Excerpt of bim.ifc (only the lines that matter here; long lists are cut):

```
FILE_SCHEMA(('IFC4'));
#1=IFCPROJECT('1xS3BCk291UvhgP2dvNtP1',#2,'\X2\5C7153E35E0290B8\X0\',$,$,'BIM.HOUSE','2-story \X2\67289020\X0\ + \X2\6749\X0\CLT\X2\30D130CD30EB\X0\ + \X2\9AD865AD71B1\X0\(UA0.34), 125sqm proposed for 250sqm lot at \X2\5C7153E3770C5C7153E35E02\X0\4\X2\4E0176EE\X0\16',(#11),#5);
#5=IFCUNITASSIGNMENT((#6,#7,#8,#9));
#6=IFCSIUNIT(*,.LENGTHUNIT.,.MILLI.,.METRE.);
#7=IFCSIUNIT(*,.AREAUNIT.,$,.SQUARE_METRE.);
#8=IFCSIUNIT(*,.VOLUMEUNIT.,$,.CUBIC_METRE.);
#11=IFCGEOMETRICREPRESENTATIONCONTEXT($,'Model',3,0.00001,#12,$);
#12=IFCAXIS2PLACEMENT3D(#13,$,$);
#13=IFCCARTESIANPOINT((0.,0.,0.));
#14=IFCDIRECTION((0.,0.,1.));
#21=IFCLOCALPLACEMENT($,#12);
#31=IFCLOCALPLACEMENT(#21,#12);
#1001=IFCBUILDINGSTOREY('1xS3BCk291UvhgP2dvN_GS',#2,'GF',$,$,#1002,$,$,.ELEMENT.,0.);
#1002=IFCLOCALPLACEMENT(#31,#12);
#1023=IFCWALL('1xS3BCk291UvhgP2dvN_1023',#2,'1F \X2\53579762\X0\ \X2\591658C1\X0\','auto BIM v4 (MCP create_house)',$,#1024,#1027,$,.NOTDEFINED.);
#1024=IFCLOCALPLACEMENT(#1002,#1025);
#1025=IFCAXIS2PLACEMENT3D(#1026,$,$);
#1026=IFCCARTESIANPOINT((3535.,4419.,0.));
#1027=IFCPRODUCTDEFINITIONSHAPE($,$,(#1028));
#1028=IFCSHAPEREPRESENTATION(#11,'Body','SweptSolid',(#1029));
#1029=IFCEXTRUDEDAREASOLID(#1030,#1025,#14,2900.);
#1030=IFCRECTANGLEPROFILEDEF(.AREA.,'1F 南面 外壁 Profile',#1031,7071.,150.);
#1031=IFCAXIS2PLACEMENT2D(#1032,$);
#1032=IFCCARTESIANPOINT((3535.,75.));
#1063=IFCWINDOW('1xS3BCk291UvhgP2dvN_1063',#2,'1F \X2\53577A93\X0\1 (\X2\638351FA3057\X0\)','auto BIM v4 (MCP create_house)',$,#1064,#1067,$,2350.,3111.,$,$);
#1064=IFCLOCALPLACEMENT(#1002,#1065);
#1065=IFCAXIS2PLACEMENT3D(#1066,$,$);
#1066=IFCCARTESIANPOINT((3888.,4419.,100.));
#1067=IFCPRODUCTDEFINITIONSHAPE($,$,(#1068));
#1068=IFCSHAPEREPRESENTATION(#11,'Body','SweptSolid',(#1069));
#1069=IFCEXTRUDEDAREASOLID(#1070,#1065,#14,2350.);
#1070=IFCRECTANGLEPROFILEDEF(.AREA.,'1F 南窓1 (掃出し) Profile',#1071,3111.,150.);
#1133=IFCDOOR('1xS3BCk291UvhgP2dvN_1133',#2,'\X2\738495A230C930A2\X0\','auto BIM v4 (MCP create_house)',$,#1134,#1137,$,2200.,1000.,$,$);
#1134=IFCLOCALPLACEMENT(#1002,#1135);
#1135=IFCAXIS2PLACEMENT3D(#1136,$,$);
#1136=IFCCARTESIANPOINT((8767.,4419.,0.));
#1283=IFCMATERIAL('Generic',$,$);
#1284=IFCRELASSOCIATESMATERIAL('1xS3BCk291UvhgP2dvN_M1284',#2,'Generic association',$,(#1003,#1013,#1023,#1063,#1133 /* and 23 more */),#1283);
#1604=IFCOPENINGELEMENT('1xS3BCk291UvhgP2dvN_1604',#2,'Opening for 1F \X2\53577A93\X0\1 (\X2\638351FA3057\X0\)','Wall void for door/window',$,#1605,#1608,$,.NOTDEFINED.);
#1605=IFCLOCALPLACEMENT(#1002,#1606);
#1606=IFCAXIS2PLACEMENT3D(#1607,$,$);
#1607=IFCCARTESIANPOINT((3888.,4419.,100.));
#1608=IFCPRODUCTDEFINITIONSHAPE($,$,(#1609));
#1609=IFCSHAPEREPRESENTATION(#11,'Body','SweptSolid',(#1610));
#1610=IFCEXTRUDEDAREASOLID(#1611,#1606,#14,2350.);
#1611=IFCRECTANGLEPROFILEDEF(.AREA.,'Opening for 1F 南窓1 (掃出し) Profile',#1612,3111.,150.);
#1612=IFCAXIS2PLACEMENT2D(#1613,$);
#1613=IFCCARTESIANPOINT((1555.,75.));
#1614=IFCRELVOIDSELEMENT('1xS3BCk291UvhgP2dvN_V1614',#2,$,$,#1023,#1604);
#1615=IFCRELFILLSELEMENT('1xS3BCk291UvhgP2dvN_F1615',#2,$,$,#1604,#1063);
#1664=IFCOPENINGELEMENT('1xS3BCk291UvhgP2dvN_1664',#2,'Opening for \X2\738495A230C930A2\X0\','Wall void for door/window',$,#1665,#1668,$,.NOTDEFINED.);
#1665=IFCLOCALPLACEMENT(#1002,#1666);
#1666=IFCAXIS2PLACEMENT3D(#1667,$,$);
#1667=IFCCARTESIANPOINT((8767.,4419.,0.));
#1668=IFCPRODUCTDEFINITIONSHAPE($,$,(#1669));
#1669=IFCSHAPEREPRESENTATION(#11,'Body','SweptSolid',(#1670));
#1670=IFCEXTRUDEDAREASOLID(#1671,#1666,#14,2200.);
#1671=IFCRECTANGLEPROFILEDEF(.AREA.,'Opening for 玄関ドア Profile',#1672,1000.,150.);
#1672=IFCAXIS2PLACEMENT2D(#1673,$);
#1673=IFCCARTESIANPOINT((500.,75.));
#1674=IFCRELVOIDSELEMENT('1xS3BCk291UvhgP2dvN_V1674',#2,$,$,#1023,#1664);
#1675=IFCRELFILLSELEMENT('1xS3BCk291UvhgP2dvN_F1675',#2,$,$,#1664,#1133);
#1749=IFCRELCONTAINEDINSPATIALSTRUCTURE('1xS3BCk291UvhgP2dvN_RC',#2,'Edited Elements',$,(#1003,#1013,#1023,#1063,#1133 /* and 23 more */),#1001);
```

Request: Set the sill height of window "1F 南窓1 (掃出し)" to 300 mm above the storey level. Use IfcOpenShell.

```python
import numpy as np
import ifcopenshell
import ifcopenshell.api.geometry
import ifcopenshell.geom
import ifcopenshell.util.element
import ifcopenshell.util.placement
import ifcopenshell.util.shape
import ifcopenshell.util.unit

model = ifcopenshell.open("bim.ifc")
unit_scale = ifcopenshell.util.unit.calculate_unit_scale(model)

window = model.by_guid("1xS3BCk291UvhgP2dvN_1063")
opening = window.FillsVoids[0].RelatingOpeningElement
storey = ifcopenshell.util.element.get_container(window, ifc_class="IfcBuildingStorey")
level = ifcopenshell.util.placement.get_local_placement(storey.ObjectPlacement)[2, 3]

# The opening's origin need not be at the sill, so measure its lowest point.
shape = ifcopenshell.geom.create_shape(ifcopenshell.geom.settings(), opening)
bottom = ifcopenshell.util.shape.get_shape_bottom_elevation(shape, shape.geometry) / unit_scale
dz = level + 0.3 / unit_scale - bottom

shift = np.array([0.0, 0.0, dz])
# The window is not placed relative to its opening, so move both.
for product in (opening, window):
    matrix = ifcopenshell.util.placement.get_local_placement(product.ObjectPlacement)
    matrix[:3, 3] += shift
    ifcopenshell.api.geometry.edit_object_placement(model, product=product, matrix=matrix, is_si=False)

print(f"moved by {dz * unit_scale:+.3f} m")

model.write("bim-out.ifc")
```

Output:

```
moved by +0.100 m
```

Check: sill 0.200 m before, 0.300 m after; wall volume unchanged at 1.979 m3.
